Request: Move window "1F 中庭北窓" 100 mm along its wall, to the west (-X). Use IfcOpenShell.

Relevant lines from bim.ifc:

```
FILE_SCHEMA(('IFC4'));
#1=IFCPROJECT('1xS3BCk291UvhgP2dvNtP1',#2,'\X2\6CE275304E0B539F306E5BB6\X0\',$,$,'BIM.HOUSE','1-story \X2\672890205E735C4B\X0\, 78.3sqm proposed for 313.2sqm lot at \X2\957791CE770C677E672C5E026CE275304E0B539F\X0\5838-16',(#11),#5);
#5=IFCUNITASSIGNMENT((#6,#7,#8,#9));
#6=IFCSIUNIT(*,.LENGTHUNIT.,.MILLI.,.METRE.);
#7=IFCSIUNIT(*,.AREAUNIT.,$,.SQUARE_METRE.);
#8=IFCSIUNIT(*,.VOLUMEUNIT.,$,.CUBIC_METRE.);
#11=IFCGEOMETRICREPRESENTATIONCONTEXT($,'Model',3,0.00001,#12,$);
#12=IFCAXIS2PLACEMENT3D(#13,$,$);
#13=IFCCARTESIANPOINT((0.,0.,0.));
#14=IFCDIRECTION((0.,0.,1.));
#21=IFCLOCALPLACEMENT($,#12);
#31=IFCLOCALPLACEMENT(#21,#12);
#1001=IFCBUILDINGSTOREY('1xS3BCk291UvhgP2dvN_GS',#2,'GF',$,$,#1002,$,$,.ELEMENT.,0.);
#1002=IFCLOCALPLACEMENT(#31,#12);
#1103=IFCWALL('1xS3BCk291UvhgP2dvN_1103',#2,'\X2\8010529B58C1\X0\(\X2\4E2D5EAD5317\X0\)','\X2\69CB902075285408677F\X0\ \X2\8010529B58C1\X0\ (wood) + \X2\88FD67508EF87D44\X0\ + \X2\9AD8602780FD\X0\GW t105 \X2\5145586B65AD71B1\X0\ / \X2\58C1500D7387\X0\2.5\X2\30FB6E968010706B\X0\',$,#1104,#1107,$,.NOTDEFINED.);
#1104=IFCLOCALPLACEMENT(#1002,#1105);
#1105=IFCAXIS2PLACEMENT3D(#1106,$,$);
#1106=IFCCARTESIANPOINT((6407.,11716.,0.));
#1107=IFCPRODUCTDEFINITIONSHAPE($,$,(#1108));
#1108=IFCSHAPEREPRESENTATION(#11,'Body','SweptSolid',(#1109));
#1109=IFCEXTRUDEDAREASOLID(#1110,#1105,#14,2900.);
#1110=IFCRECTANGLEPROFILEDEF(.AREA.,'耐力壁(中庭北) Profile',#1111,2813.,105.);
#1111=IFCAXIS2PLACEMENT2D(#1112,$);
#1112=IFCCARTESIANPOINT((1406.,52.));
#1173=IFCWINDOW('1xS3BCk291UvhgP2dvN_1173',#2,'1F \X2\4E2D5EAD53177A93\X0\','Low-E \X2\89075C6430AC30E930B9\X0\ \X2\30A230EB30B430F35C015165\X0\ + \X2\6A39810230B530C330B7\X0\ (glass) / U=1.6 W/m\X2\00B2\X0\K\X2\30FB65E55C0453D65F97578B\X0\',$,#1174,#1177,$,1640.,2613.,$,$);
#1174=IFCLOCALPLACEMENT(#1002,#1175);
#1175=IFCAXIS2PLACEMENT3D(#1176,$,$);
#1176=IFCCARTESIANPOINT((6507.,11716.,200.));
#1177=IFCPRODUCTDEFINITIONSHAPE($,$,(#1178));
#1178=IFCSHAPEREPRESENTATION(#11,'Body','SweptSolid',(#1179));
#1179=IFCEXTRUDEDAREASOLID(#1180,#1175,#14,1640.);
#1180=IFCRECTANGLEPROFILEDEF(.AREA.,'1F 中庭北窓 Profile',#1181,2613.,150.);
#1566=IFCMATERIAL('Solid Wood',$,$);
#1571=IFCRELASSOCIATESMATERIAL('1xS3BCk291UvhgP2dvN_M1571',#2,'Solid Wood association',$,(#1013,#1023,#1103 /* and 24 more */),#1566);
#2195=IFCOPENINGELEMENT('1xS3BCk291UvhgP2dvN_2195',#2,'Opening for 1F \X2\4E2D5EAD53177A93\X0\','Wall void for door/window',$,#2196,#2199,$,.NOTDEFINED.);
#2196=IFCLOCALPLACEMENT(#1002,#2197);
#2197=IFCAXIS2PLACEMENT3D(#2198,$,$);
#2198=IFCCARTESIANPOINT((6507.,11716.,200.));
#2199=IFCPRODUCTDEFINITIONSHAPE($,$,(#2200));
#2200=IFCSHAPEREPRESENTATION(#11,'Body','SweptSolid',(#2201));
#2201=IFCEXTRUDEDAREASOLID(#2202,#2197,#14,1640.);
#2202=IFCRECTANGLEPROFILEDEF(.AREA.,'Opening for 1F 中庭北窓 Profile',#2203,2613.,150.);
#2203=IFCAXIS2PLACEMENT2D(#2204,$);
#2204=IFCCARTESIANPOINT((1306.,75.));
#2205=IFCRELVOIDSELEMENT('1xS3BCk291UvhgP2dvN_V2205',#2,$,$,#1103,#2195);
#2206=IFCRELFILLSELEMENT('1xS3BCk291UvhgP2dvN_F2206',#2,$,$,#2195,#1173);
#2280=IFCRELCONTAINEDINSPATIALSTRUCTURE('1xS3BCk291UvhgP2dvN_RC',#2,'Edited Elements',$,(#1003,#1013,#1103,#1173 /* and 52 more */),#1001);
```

```python
import ifcopenshell
import ifcopenshell.api.geometry
import ifcopenshell.util.placement

model = ifcopenshell.open("bim.ifc")

window = model.by_guid("1xS3BCk291UvhgP2dvN_1173")
opening = window.FillsVoids[0].RelatingOpeningElement
wall = opening.VoidsElements[0].RelatingBuildingElement

wall_matrix = ifcopenshell.util.placement.get_local_placement(wall.ObjectPlacement)
shift = wall_matrix[:3, 0] * -100.0
before = ifcopenshell.util.placement.get_local_placement(window.ObjectPlacement)[:3, 3].copy()

# The window is not placed relative to its opening, so move both.
for product in (opening, window):
    matrix = ifcopenshell.util.placement.get_local_placement(product.ObjectPlacement)
    matrix[:3, 3] += shift
    ifcopenshell.api.geometry.edit_object_placement(model, product=product, matrix=matrix, is_si=False)

after = ifcopenshell.util.placement.get_local_placement(window.ObjectPlacement)[:3, 3]
print("window moved by", (after - before).round(3) + 0.0)

model.write("bim_v2.ifc")
```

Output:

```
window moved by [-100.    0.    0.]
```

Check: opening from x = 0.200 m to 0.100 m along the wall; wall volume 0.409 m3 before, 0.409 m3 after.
